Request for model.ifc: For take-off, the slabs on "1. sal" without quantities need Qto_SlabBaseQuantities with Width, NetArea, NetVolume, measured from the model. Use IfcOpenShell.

First a look at what the model holds.

```python
import ifcopenshell
import ifcopenshell.util.element
import ifcopenshell.util.unit

model = ifcopenshell.open("model.ifc")
print(model.schema)
for unit_type in ("LENGTHUNIT", "AREAUNIT", "VOLUMEUNIT"):
    print(unit_type, ifcopenshell.util.unit.calculate_unit_scale(model, unit_type))
storey = next(s for s in model.by_type("IfcBuildingStorey") if s.Name == "1. sal")
slabs = [e for e in ifcopenshell.util.element.get_decomposition(storey) if e.is_a("IfcSlab")]
for e in sorted(slabs, key=lambda e: e.id()):
    print(e.id(), e.is_a(), e.Name, list(ifcopenshell.util.element.get_psets(e, qtos_only=True)), sep=" | ")
```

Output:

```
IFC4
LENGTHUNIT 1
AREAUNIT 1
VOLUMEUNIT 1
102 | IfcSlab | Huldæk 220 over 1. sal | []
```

```python
import ifcopenshell
import ifcopenshell.api.pset
import ifcopenshell.geom
import ifcopenshell.util.element
import ifcopenshell.util.shape
import ifcopenshell.util.unit

model = ifcopenshell.open("model.ifc")
unit_scale = ifcopenshell.util.unit.calculate_unit_scale(model)
area_scale = ifcopenshell.util.unit.calculate_unit_scale(model, "AREAUNIT")
volume_scale = ifcopenshell.util.unit.calculate_unit_scale(model, "VOLUMEUNIT")
settings = ifcopenshell.geom.settings()

storey = next(s for s in model.by_type("IfcBuildingStorey") if s.Name == "1. sal")
slabs = [e for e in ifcopenshell.util.element.get_decomposition(storey) if e.is_a("IfcSlab")]

for e in sorted(slabs, key=lambda e: e.id()):
    if ifcopenshell.util.element.get_psets(e, qtos_only=True, should_inherit=False):
        continue
    # Geometry comes back in metres, in the element's own axes.
    shape = ifcopenshell.geom.create_shape(settings, e)
    values = {
        "Width": ifcopenshell.util.shape.get_z(shape.geometry) / unit_scale,
        "NetArea": ifcopenshell.util.shape.get_footprint_area(shape.geometry) / area_scale,
        "NetVolume": ifcopenshell.util.shape.get_volume(shape.geometry) / volume_scale,
    }
    qto = ifcopenshell.api.pset.add_qto(model, product=e, name="Qto_SlabBaseQuantities")
    ifcopenshell.api.pset.edit_qto(model, qto=qto, properties=values)
    print(e.id(), {k: round(v, 3) for k, v in values.items()})

model.write("model_edited.ifc")
```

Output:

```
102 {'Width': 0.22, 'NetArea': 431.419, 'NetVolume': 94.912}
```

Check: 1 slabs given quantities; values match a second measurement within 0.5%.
